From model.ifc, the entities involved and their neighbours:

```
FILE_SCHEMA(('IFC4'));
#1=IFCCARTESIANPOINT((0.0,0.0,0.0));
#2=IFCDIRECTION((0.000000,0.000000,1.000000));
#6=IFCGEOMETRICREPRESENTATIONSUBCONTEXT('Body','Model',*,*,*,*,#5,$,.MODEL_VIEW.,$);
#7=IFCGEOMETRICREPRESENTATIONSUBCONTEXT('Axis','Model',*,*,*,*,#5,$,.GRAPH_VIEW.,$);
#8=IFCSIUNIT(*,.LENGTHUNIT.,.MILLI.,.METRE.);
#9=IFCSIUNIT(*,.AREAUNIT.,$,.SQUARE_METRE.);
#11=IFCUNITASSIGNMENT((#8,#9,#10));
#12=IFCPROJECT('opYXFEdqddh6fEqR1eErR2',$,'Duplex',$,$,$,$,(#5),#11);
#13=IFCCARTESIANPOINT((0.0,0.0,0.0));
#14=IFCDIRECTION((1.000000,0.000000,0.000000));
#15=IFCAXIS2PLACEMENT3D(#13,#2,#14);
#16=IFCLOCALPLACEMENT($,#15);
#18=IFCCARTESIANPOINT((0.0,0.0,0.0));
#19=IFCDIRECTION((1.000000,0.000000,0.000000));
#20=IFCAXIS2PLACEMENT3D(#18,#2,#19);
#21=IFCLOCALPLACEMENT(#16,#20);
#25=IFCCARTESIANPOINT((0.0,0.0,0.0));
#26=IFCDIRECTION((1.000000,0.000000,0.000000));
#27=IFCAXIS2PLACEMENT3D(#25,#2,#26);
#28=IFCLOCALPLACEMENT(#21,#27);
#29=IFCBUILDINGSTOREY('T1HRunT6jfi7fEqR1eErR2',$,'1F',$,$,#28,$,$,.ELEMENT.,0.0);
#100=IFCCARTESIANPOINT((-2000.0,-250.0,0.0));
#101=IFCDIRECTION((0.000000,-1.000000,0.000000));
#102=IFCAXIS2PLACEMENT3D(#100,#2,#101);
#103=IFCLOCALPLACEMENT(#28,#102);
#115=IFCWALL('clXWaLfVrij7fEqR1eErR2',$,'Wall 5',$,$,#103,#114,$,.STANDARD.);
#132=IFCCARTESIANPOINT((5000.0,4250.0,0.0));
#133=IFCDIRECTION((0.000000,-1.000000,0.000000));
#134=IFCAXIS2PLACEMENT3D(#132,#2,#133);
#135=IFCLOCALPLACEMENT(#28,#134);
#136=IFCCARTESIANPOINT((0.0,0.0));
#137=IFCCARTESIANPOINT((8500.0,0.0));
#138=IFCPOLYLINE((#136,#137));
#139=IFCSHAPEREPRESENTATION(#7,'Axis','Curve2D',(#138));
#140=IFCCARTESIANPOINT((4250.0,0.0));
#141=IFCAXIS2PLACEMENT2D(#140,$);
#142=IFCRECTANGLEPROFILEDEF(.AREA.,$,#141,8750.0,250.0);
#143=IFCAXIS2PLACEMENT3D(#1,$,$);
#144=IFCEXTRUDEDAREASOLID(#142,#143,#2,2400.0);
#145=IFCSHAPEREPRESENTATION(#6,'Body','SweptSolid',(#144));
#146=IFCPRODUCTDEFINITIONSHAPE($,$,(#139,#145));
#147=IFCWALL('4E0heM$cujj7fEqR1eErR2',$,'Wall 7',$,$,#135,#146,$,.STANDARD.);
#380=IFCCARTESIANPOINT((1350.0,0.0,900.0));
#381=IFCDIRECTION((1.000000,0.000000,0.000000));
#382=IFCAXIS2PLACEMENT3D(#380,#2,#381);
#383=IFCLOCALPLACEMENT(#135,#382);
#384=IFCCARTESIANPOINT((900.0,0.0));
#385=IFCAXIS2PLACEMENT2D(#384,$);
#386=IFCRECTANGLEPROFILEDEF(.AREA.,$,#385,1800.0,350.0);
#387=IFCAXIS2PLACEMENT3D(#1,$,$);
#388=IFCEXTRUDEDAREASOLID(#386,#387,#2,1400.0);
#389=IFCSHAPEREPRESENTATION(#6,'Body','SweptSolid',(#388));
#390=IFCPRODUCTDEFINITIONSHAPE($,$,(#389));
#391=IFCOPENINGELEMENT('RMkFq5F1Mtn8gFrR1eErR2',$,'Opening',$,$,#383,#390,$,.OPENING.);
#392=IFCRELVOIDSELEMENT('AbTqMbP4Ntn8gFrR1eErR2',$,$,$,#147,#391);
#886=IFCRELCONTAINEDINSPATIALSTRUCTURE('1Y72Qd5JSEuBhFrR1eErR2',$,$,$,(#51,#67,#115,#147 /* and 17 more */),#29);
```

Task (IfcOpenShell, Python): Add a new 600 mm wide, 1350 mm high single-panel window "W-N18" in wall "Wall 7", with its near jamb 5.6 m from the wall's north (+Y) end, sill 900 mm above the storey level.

```python
import numpy as np
import ifcopenshell
import ifcopenshell.api.feature
import ifcopenshell.api.geometry
import ifcopenshell.api.root
import ifcopenshell.api.spatial
import ifcopenshell.geom
import ifcopenshell.util.element
import ifcopenshell.util.placement
import ifcopenshell.util.representation
import ifcopenshell.util.shape
import ifcopenshell.util.unit

model = ifcopenshell.open("model.ifc")
unit_scale = ifcopenshell.util.unit.calculate_unit_scale(model)
settings = ifcopenshell.geom.settings()


def volume(element):
    """Net volume in cubic metres, openings subtracted."""
    shape = ifcopenshell.geom.create_shape(settings, element)
    return ifcopenshell.util.shape.get_volume(shape.geometry)


wall = model.by_guid("4E0heM$cujj7fEqR1eErR2")
storey = ifcopenshell.util.element.get_container(wall, ifc_class="IfcBuildingStorey")
context = ifcopenshell.util.representation.get_context(model, "Model", "Body", "MODEL_VIEW")
before = volume(wall)

width, height, from_end, sill = 0.6, 1.35, 5.6, 0.9  # metres

# The wall runs along its own X axis, and the end named is its -X end.
wall_shape = ifcopenshell.geom.create_shape(settings, wall)
x, y, z = ifcopenshell.util.shape.get_vertices(wall_shape.geometry).T
start = x.min() + from_end
face, thickness = float(y.min()), float(y.max() - y.min())
wall_matrix = ifcopenshell.util.placement.get_local_placement(wall.ObjectPlacement)
level = ifcopenshell.util.placement.get_local_placement(storey.ObjectPlacement)[2, 3]


def in_wall(x, y):
    """Placement at x, y metres in the wall's axes, at sill height."""
    matrix = wall_matrix.copy()
    matrix[:, 3] = wall_matrix @ np.array([x / unit_scale, y / unit_scale, 0.0, 1.0])
    matrix[2, 3] = level + sill / unit_scale
    return matrix


# Opening: a box that overshoots both wall faces by 50 mm.
opening = ifcopenshell.api.root.create_entity(model, ifc_class="IfcOpeningElement", predefined_type="OPENING")
box = ifcopenshell.api.geometry.add_wall_representation(
    model, context=context, length=width, height=height, thickness=thickness + 0.1
)
ifcopenshell.api.geometry.assign_representation(model, product=opening, representation=box)
ifcopenshell.api.geometry.edit_object_placement(model, product=opening, matrix=in_wall(start, face - 0.05), is_si=False)
ifcopenshell.api.feature.add_feature(model, feature=opening, element=wall)

window = ifcopenshell.api.root.create_entity(model, ifc_class="IfcWindow", name="W-N18", predefined_type="WINDOW")
window.OverallWidth, window.OverallHeight = width / unit_scale, height / unit_scale
window.PartitioningType = "SINGLE_PANEL"
body = ifcopenshell.api.geometry.add_window_representation(
    model,
    context=context,
    overall_width=window.OverallWidth,
    overall_height=window.OverallHeight,
    partition_type="SINGLE_PANEL",
)
ifcopenshell.api.geometry.assign_representation(model, product=window, representation=body)
ifcopenshell.api.spatial.assign_container(model, products=[window], relating_structure=storey)
ifcopenshell.api.feature.add_filling(model, opening=opening, element=window)

# Centre the window in the wall's thickness.
ifcopenshell.api.geometry.edit_object_placement(model, product=window, matrix=in_wall(start, face), is_si=False)
window_shape = ifcopenshell.geom.create_shape(settings, window)
depth = ifcopenshell.util.shape.get_vertices(window_shape.geometry)[:, 1]
offset = face + thickness / 2 - (depth.min() + depth.max()) / 2
ifcopenshell.api.geometry.edit_object_placement(model, product=window, matrix=in_wall(start, offset), is_si=False)

after = volume(wall)

print(f"wall volume {before:.3f} -> {after:.3f} m3")

model.write("model_updated.ifc")
```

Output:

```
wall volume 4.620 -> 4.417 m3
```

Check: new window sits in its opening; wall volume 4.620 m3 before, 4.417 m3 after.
